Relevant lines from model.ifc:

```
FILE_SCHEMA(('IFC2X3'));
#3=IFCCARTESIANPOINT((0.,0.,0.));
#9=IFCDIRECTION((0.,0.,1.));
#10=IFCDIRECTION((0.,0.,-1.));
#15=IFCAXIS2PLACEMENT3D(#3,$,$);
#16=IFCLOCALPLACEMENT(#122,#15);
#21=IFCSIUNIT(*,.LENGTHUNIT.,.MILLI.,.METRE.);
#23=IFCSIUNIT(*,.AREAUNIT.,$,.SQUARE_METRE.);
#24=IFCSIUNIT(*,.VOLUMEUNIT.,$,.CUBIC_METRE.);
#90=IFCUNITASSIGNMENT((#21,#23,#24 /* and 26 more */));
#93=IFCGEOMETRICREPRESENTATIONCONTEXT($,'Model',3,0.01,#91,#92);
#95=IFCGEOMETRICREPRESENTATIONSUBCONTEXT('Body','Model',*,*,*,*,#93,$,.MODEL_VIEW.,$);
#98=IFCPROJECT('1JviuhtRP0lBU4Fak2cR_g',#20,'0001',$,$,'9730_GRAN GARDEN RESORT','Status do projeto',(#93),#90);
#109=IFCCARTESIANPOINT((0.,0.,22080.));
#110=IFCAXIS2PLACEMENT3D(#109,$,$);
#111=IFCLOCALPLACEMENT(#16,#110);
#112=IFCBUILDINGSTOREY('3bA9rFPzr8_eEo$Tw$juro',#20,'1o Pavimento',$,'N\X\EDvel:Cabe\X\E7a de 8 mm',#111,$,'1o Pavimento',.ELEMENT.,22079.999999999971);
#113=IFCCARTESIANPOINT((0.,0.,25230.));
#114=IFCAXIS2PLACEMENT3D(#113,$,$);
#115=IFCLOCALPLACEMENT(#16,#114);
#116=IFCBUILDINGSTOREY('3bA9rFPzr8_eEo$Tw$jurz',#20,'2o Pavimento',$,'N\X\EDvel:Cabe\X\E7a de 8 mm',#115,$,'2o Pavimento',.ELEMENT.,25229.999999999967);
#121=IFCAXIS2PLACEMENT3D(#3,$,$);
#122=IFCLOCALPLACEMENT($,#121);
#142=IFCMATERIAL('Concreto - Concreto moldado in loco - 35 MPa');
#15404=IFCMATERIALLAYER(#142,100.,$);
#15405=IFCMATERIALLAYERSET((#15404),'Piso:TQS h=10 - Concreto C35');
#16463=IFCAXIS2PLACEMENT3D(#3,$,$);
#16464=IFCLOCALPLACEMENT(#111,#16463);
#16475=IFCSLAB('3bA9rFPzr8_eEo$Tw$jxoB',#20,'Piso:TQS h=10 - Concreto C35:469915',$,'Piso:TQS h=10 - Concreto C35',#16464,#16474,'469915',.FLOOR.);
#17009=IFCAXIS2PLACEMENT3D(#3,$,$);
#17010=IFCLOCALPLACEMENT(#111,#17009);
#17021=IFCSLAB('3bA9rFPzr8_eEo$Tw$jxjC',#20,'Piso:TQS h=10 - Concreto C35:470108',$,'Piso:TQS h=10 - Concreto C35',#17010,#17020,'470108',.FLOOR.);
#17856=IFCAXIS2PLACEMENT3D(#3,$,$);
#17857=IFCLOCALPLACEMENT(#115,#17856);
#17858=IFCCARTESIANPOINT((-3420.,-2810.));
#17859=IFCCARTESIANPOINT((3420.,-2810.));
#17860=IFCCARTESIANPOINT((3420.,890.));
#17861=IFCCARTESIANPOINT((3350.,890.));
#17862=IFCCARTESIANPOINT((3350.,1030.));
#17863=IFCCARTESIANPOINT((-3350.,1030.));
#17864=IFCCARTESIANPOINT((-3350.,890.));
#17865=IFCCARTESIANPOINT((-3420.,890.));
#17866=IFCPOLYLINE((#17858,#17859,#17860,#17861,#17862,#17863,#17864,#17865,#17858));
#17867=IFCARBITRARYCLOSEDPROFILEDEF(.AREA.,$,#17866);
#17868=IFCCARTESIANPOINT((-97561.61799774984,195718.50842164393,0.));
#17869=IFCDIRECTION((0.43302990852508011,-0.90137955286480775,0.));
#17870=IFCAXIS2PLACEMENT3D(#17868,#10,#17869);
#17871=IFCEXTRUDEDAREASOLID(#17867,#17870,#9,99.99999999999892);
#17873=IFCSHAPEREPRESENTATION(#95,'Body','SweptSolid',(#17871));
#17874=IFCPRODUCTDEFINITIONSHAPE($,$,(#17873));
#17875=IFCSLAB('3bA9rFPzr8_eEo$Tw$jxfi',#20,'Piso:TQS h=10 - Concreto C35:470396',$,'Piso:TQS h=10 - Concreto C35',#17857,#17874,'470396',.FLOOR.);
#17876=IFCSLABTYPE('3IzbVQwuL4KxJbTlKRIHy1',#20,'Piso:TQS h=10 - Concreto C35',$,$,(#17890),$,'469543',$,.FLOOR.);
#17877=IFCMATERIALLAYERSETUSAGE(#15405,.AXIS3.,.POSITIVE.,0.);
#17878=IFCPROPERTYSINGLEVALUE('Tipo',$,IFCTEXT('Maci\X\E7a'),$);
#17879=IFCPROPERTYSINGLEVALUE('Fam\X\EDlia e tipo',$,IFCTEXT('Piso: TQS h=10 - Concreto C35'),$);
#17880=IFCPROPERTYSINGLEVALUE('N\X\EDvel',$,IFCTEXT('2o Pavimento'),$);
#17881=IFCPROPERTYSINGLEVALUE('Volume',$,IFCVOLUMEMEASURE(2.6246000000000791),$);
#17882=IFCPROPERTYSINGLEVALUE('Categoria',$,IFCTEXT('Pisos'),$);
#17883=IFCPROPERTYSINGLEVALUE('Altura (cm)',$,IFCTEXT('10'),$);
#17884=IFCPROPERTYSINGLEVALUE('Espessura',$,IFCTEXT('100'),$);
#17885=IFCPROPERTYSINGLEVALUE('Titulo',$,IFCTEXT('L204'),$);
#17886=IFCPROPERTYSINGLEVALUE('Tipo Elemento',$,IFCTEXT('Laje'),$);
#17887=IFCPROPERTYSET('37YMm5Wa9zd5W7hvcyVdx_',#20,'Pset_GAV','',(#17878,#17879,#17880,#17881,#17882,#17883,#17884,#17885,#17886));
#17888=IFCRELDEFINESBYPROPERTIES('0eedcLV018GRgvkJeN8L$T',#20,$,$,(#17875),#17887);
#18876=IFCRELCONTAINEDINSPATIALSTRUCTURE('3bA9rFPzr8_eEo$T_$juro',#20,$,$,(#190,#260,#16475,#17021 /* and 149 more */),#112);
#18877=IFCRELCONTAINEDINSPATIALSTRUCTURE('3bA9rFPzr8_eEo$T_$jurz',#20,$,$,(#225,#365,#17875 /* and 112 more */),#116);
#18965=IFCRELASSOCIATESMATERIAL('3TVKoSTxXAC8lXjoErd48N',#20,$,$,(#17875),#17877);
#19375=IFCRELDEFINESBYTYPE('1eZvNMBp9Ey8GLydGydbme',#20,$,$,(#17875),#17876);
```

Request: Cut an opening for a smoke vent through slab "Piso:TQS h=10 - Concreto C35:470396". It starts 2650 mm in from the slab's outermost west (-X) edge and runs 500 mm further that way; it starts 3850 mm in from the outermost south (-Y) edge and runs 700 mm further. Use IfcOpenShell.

```python
import numpy as np
import ifcopenshell
import ifcopenshell.api.feature
import ifcopenshell.api.geometry
import ifcopenshell.api.pset
import ifcopenshell.api.root
import ifcopenshell.geom
import ifcopenshell.util.element
import ifcopenshell.util.placement
import ifcopenshell.util.representation
import ifcopenshell.util.shape
import ifcopenshell.util.unit

model = ifcopenshell.open("model.ifc")
unit_scale = ifcopenshell.util.unit.calculate_unit_scale(model)
volume_scale = ifcopenshell.util.unit.calculate_unit_scale(model, "VOLUMEUNIT")
settings = ifcopenshell.geom.settings()


def volume(element):
    """Net volume in cubic metres, openings subtracted."""
    shape = ifcopenshell.geom.create_shape(settings, element)
    return ifcopenshell.util.shape.get_volume(shape.geometry)


slab = model.by_guid("3bA9rFPzr8_eEo$Tw$jxfi")
before = volume(slab)

# Extent in the slab's own axes, in metres. The edges named are its -X and -Y sides.
slab_shape = ifcopenshell.geom.create_shape(settings, slab)
vertices = ifcopenshell.util.shape.get_vertices(slab_shape.geometry)
x_min, y_min, bottom = vertices.min(axis=0)
top = vertices[:, 2].max()

opening = ifcopenshell.api.root.create_entity(model, ifc_class="IfcOpeningElement", name="Smoke vent opening")
context = ifcopenshell.util.representation.get_context(model, "Model", "Body", "MODEL_VIEW")
width, depth = 0.5, 0.7
outline = [(0.0, 0.0), (width, 0.0), (width, depth), (0.0, depth), (0.0, 0.0)]
# Overshoot both faces by 50 mm so the cut is clean.
shape = ifcopenshell.api.geometry.add_slab_representation(
    model, context=context, depth=top - bottom + 0.1, polyline=outline
)
ifcopenshell.api.geometry.assign_representation(model, product=opening, representation=shape)

matrix = ifcopenshell.util.placement.get_local_placement(slab.ObjectPlacement)
matrix[:, 3] = matrix @ np.append(np.array([x_min + 2.65, y_min + 3.85, bottom - 0.05]) / unit_scale, 1.0)
ifcopenshell.api.geometry.edit_object_placement(model, product=opening, matrix=matrix, is_si=False)
ifcopenshell.api.feature.add_feature(model, feature=opening, element=slab)

after = volume(slab)

# Update the slab's stored quantities.
pset = model.by_id(ifcopenshell.util.element.get_pset(slab, "Pset_GAV", should_inherit=False)["id"])
ifcopenshell.api.pset.edit_pset(model, pset=pset, properties={
    "Volume": model.create_entity("IfcVolumeMeasure", after / volume_scale),
})

print(f"slab volume {before:.3f} -> {after:.3f} m3")

model.write("model_v2.ifc")
```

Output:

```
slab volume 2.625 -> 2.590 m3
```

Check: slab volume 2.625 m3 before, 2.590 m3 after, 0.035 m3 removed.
